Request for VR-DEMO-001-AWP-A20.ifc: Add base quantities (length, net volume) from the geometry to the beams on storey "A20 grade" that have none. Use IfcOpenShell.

First a look at what the model holds.

```python
import ifcopenshell
import ifcopenshell.util.element
import ifcopenshell.util.unit

model = ifcopenshell.open("VR-DEMO-001-AWP-A20.ifc")
print(model.schema)
for unit_type in ("LENGTHUNIT", "AREAUNIT", "VOLUMEUNIT"):
    print(unit_type, ifcopenshell.util.unit.calculate_unit_scale(model, unit_type))
storey = next(s for s in model.by_type("IfcBuildingStorey") if s.Name == "A20 grade")
beams = [e for e in ifcopenshell.util.element.get_decomposition(storey) if e.is_a("IfcBeam")]
for e in sorted(beams, key=lambda e: e.id()):
    print(e.id(), e.is_a(), e.Name, list(ifcopenshell.util.element.get_psets(e, qtos_only=True)), sep=" | ")
```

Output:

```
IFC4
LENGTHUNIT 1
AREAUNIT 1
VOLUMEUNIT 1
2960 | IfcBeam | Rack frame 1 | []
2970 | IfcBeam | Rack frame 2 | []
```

```python
import ifcopenshell
import ifcopenshell.api.pset
import ifcopenshell.geom
import ifcopenshell.util.element
import ifcopenshell.util.shape
import ifcopenshell.util.unit

model = ifcopenshell.open("VR-DEMO-001-AWP-A20.ifc")
unit_scale = ifcopenshell.util.unit.calculate_unit_scale(model)
volume_scale = ifcopenshell.util.unit.calculate_unit_scale(model, "VOLUMEUNIT")
settings = ifcopenshell.geom.settings()

storey = next(s for s in model.by_type("IfcBuildingStorey") if s.Name == "A20 grade")
beams = [e for e in ifcopenshell.util.element.get_decomposition(storey) if e.is_a("IfcBeam")]

for e in sorted(beams, key=lambda e: e.id()):
    if ifcopenshell.util.element.get_psets(e, qtos_only=True, should_inherit=False):
        continue
    # Geometry comes back in metres, in the element's own axes.
    shape = ifcopenshell.geom.create_shape(settings, e)
    values = {
        "Length": ifcopenshell.util.shape.get_max_xyz(shape.geometry) / unit_scale,
        "NetVolume": ifcopenshell.util.shape.get_volume(shape.geometry) / volume_scale,
    }
    qto = ifcopenshell.api.pset.add_qto(model, product=e, name="Qto_BeamBaseQuantities")
    ifcopenshell.api.pset.edit_qto(model, qto=qto, properties=values)
    print(e.id(), {k: round(v, 3) for k, v in values.items()})

model.write("VR-DEMO-001-AWP-A20_rev.ifc")
```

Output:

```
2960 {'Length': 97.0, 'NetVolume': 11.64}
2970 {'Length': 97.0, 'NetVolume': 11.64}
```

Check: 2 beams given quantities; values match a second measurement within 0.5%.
